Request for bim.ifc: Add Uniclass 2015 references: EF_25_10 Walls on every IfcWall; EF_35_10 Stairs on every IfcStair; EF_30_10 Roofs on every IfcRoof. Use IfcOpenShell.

First a look at what the model holds.

```python
import ifcopenshell

model = ifcopenshell.open("bim.ifc")
print(model.schema)
print("classifications:", [c.Name for c in model.by_type("IfcClassification")])
for ifc_class in ("IfcDoor", "IfcRoof", "IfcStair", "IfcWall", "IfcWindow"):
    print(ifc_class, len(model.by_type(ifc_class)))
```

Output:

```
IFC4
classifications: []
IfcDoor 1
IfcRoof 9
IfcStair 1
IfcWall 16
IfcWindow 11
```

```python
import ifcopenshell
import ifcopenshell.api.classification

model = ifcopenshell.open("bim.ifc")

system = ifcopenshell.api.classification.add_classification(model, classification="Uniclass 2015")

codes = {
    "IfcWall": ("EF_25_10", "Walls"),
    "IfcStair": ("EF_35_10", "Stairs"),
    "IfcRoof": ("EF_30_10", "Roofs"),
}
for ifc_class, (code, name) in codes.items():
    products = model.by_type(ifc_class)
    ifcopenshell.api.classification.add_reference(
        model, products=products, classification=system, identification=code, name=name
    )
    print(code, len(products))

model.write("bim_v2.ifc")
```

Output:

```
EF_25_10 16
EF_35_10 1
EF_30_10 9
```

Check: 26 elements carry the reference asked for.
